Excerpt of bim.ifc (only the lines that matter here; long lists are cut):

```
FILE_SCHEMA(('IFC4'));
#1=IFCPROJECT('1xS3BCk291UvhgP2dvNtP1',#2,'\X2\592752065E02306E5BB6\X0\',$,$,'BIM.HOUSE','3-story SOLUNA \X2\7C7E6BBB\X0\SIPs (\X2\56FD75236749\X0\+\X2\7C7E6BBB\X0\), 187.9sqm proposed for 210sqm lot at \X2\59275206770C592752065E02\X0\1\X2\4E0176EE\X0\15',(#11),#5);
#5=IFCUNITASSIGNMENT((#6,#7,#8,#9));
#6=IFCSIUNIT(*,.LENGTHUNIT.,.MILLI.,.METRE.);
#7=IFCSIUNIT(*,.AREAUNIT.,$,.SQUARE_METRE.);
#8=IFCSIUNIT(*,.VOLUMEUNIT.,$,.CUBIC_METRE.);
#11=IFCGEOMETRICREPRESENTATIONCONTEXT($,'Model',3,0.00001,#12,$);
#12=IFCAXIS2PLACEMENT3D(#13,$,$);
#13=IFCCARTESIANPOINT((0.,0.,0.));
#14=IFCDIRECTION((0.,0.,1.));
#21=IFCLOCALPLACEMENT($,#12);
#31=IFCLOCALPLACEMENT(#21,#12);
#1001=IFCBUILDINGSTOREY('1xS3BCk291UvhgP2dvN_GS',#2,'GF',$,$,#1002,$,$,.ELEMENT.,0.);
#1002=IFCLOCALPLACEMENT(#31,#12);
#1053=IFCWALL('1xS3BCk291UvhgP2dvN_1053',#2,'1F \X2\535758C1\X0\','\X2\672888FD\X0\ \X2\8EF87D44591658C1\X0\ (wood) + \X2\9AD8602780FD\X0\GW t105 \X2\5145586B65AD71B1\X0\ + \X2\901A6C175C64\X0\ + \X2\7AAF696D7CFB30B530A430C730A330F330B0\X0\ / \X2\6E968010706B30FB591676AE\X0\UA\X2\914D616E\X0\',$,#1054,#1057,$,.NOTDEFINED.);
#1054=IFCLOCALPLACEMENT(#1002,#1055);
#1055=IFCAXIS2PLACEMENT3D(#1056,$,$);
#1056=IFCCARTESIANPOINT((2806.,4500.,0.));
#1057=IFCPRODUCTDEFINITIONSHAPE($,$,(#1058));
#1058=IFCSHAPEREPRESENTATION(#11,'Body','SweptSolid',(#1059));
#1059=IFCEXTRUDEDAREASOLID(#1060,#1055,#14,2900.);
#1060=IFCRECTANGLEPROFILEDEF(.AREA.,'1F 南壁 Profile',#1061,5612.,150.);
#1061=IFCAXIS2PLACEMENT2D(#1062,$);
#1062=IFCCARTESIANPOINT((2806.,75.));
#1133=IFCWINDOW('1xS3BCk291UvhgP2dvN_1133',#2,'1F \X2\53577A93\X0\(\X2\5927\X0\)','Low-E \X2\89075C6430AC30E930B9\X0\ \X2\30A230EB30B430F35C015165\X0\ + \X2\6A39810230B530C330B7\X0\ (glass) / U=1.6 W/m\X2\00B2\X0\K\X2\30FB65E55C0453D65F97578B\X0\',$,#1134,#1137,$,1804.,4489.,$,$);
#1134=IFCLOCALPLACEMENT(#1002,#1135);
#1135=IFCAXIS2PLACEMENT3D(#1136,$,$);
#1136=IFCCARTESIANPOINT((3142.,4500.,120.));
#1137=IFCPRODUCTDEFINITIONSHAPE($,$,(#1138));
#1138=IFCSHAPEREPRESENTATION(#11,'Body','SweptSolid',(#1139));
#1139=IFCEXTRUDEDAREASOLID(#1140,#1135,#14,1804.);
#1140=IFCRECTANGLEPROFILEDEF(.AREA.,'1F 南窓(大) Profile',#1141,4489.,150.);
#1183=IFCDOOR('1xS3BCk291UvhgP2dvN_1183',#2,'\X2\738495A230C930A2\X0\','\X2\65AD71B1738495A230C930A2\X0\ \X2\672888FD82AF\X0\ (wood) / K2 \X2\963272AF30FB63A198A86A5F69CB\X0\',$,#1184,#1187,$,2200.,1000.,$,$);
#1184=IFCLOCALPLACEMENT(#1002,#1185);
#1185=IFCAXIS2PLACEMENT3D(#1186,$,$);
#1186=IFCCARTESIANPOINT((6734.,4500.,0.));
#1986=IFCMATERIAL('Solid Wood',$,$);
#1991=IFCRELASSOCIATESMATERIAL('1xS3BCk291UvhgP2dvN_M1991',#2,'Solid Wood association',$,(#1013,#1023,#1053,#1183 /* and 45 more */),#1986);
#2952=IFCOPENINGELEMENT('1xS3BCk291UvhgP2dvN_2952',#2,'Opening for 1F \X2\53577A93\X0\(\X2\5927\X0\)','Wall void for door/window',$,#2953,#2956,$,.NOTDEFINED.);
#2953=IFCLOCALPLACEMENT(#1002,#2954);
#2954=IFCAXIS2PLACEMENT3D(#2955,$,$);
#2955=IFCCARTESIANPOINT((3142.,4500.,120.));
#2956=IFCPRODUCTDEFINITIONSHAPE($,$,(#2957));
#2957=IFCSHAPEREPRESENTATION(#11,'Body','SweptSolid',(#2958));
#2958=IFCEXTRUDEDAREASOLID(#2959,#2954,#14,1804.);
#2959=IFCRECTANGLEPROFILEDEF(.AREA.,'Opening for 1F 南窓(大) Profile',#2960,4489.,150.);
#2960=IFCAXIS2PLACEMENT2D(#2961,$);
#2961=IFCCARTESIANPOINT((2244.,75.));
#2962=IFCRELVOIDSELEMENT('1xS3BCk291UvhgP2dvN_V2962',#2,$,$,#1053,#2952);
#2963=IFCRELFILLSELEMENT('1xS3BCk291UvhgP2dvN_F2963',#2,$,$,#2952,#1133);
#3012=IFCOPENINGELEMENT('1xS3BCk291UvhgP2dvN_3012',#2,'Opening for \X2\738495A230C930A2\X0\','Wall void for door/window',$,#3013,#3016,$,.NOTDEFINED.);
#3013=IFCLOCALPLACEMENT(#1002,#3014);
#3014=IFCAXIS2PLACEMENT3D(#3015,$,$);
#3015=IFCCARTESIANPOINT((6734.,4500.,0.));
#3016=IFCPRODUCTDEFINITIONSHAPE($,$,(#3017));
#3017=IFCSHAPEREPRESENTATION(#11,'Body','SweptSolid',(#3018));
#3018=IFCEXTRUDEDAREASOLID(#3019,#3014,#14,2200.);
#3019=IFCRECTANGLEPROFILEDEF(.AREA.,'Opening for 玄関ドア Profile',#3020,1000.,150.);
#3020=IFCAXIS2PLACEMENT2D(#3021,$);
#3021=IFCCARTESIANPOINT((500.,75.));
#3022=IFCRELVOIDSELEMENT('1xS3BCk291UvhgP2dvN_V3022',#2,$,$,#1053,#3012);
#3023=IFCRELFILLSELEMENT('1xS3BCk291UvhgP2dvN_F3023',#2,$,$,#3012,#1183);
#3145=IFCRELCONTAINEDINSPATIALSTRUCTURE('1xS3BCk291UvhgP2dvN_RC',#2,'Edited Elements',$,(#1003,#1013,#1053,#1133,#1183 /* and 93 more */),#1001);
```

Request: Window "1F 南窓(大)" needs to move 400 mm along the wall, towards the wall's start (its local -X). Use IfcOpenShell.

```python
import ifcopenshell
import ifcopenshell.api.geometry
import ifcopenshell.util.placement
import ifcopenshell.util.unit

model = ifcopenshell.open("bim.ifc")
unit_scale = ifcopenshell.util.unit.calculate_unit_scale(model)

window = model.by_guid("1xS3BCk291UvhgP2dvN_1133")
opening = window.FillsVoids[0].RelatingOpeningElement
wall = opening.VoidsElements[0].RelatingBuildingElement

wall_matrix = ifcopenshell.util.placement.get_local_placement(wall.ObjectPlacement)
shift = wall_matrix[:3, 0] * -0.4 / unit_scale
before = ifcopenshell.util.placement.get_local_placement(window.ObjectPlacement)[:3, 3].copy()

# The window is not placed relative to its opening, so move both.
for product in (opening, window):
    matrix = ifcopenshell.util.placement.get_local_placement(product.ObjectPlacement)
    matrix[:3, 3] += shift
    ifcopenshell.api.geometry.edit_object_placement(model, product=product, matrix=matrix, is_si=False)

after = ifcopenshell.util.placement.get_local_placement(window.ObjectPlacement)[:3, 3]
print("window moved by", (after - before).round(3) + 0.0)

model.write("bim_updated.ifc")
```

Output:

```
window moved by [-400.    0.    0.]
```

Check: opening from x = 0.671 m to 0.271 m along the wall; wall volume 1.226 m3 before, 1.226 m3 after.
